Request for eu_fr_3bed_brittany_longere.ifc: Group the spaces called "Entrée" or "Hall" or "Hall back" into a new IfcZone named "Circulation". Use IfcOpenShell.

First a look at what the model holds.

```python
import ifcopenshell

model = ifcopenshell.open("eu_fr_3bed_brittany_longere.ifc")
print(model.schema)
seen = {}
for space in model.by_type("IfcSpace"):
    seen[space.LongName] = seen.get(space.LongName, 0) + 1
for name, count in sorted(seen.items(), key=str):
    print(count, "x", name)
print("zones:", [z.Name for z in model.by_type("IfcZone")][:20])
```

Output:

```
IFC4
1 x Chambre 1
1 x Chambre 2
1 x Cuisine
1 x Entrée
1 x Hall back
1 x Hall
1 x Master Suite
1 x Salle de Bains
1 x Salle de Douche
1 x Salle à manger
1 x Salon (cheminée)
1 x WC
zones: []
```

```python
import ifcopenshell
import ifcopenshell.api.group
import ifcopenshell.api.root

model = ifcopenshell.open("eu_fr_3bed_brittany_longere.ifc")

names = {"Entrée", "Hall", "Hall back"}
spaces = [s for s in model.by_type("IfcSpace") if s.LongName in names]

zone = ifcopenshell.api.root.create_entity(model, ifc_class="IfcZone", name="Circulation")
ifcopenshell.api.group.assign_group(model, products=spaces, group=zone)
print(len(spaces), "spaces in", zone.Name)

model.write("eu_fr_3bed_brittany_longere_edited.ifc")
```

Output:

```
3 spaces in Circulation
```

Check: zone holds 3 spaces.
